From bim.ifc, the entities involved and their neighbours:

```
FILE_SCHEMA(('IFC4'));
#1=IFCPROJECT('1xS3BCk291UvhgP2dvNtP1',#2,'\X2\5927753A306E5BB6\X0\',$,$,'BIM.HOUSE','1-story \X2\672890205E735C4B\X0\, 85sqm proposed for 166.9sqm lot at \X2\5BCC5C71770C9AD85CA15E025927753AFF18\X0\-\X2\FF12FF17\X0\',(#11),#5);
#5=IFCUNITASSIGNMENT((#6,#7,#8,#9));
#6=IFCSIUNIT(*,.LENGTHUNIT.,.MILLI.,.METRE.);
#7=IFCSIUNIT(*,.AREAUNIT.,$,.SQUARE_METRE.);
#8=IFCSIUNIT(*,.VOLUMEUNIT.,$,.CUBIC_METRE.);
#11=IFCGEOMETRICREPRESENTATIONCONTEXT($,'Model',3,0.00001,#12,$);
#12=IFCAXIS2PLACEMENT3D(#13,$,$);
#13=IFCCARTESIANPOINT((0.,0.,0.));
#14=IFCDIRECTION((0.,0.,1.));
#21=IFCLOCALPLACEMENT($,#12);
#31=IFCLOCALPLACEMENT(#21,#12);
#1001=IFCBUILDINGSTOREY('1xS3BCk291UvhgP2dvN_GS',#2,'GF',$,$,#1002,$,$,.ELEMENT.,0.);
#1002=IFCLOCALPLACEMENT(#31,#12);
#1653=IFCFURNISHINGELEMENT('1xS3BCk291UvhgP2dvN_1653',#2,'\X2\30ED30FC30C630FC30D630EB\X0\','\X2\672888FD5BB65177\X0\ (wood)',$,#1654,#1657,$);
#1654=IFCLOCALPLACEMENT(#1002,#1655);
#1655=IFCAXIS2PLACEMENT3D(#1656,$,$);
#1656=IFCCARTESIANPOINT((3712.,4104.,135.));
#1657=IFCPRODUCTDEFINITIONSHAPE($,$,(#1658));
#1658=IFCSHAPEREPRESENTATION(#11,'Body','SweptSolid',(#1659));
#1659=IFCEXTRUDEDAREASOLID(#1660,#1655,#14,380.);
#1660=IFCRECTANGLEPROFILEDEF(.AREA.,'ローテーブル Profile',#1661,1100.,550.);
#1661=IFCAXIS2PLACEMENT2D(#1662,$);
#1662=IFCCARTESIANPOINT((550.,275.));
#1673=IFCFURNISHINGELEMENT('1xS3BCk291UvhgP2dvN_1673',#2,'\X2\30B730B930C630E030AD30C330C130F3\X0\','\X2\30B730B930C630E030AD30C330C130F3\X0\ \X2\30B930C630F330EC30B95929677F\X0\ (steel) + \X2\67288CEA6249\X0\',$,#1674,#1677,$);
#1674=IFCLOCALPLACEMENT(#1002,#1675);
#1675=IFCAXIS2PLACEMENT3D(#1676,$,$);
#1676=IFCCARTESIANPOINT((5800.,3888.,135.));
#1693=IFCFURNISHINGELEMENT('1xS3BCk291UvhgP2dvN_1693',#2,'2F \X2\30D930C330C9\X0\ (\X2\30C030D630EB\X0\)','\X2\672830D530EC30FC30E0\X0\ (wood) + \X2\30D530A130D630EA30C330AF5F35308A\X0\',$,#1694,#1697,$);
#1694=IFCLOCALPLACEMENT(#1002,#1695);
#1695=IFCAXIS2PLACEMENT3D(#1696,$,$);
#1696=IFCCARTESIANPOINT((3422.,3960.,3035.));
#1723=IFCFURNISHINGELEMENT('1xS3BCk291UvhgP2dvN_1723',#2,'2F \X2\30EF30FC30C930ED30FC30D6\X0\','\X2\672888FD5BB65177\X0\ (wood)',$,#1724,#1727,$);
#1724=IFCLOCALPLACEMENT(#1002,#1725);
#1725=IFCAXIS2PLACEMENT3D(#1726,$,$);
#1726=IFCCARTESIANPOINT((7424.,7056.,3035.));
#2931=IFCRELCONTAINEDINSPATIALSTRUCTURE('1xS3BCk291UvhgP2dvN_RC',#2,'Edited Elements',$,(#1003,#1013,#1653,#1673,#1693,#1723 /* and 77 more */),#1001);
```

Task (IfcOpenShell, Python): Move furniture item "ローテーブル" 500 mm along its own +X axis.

```python
import ifcopenshell
import ifcopenshell.api.geometry
import ifcopenshell.util.placement
import ifcopenshell.util.unit

model = ifcopenshell.open("bim.ifc")
unit_scale = ifcopenshell.util.unit.calculate_unit_scale(model)

item = model.by_guid("1xS3BCk291UvhgP2dvN_1653")
matrix = ifcopenshell.util.placement.get_local_placement(item.ObjectPlacement)
matrix[:3, 3] += matrix[:3, 0] * 0.5 / unit_scale
ifcopenshell.api.geometry.edit_object_placement(model, product=item, matrix=matrix, is_si=False)

print(ifcopenshell.util.placement.get_local_placement(item.ObjectPlacement).round(3) + 0.0)

model.write("bim_updated.ifc")
```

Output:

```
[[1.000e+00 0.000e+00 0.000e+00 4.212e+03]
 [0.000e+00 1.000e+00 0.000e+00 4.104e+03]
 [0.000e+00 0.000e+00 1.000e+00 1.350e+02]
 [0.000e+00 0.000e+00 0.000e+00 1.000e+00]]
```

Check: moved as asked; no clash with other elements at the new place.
